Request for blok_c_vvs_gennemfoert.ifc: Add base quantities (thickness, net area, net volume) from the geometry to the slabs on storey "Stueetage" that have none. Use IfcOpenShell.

First a look at what the model holds.

```python
import ifcopenshell
import ifcopenshell.util.element
import ifcopenshell.util.unit

model = ifcopenshell.open("blok_c_vvs_gennemfoert.ifc")
print(model.schema)
for unit_type in ("LENGTHUNIT", "AREAUNIT", "VOLUMEUNIT"):
    print(unit_type, ifcopenshell.util.unit.calculate_unit_scale(model, unit_type))
storey = next(s for s in model.by_type("IfcBuildingStorey") if s.Name == "Stueetage")
slabs = [e for e in ifcopenshell.util.element.get_decomposition(storey) if e.is_a("IfcSlab")]
for e in sorted(slabs, key=lambda e: e.id()):
    print(e.id(), e.is_a(), e.Name, list(ifcopenshell.util.element.get_psets(e, qtos_only=True)), sep=" | ")
```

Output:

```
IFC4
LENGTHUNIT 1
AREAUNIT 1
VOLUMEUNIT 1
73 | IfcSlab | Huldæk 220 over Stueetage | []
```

```python
import ifcopenshell
import ifcopenshell.api.pset
import ifcopenshell.geom
import ifcopenshell.util.element
import ifcopenshell.util.shape
import ifcopenshell.util.unit

model = ifcopenshell.open("blok_c_vvs_gennemfoert.ifc")
unit_scale = ifcopenshell.util.unit.calculate_unit_scale(model)
area_scale = ifcopenshell.util.unit.calculate_unit_scale(model, "AREAUNIT")
volume_scale = ifcopenshell.util.unit.calculate_unit_scale(model, "VOLUMEUNIT")
settings = ifcopenshell.geom.settings()

storey = next(s for s in model.by_type("IfcBuildingStorey") if s.Name == "Stueetage")
slabs = [e for e in ifcopenshell.util.element.get_decomposition(storey) if e.is_a("IfcSlab")]

for e in sorted(slabs, key=lambda e: e.id()):
    if ifcopenshell.util.element.get_psets(e, qtos_only=True, should_inherit=False):
        continue
    # Geometry comes back in metres, in the element's own axes.
    shape = ifcopenshell.geom.create_shape(settings, e)
    values = {
        "Width": ifcopenshell.util.shape.get_z(shape.geometry) / unit_scale,
        "NetArea": ifcopenshell.util.shape.get_footprint_area(shape.geometry) / area_scale,
        "NetVolume": ifcopenshell.util.shape.get_volume(shape.geometry) / volume_scale,
    }
    qto = ifcopenshell.api.pset.add_qto(model, product=e, name="Qto_SlabBaseQuantities")
    ifcopenshell.api.pset.edit_qto(model, qto=qto, properties=values)
    print(e.id(), {k: round(v, 3) for k, v in values.items()})

model.write("blok_c_vvs_gennemfoert_updated.ifc")
```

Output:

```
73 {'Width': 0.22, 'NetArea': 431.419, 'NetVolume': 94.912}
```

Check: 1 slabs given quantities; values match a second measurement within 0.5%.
